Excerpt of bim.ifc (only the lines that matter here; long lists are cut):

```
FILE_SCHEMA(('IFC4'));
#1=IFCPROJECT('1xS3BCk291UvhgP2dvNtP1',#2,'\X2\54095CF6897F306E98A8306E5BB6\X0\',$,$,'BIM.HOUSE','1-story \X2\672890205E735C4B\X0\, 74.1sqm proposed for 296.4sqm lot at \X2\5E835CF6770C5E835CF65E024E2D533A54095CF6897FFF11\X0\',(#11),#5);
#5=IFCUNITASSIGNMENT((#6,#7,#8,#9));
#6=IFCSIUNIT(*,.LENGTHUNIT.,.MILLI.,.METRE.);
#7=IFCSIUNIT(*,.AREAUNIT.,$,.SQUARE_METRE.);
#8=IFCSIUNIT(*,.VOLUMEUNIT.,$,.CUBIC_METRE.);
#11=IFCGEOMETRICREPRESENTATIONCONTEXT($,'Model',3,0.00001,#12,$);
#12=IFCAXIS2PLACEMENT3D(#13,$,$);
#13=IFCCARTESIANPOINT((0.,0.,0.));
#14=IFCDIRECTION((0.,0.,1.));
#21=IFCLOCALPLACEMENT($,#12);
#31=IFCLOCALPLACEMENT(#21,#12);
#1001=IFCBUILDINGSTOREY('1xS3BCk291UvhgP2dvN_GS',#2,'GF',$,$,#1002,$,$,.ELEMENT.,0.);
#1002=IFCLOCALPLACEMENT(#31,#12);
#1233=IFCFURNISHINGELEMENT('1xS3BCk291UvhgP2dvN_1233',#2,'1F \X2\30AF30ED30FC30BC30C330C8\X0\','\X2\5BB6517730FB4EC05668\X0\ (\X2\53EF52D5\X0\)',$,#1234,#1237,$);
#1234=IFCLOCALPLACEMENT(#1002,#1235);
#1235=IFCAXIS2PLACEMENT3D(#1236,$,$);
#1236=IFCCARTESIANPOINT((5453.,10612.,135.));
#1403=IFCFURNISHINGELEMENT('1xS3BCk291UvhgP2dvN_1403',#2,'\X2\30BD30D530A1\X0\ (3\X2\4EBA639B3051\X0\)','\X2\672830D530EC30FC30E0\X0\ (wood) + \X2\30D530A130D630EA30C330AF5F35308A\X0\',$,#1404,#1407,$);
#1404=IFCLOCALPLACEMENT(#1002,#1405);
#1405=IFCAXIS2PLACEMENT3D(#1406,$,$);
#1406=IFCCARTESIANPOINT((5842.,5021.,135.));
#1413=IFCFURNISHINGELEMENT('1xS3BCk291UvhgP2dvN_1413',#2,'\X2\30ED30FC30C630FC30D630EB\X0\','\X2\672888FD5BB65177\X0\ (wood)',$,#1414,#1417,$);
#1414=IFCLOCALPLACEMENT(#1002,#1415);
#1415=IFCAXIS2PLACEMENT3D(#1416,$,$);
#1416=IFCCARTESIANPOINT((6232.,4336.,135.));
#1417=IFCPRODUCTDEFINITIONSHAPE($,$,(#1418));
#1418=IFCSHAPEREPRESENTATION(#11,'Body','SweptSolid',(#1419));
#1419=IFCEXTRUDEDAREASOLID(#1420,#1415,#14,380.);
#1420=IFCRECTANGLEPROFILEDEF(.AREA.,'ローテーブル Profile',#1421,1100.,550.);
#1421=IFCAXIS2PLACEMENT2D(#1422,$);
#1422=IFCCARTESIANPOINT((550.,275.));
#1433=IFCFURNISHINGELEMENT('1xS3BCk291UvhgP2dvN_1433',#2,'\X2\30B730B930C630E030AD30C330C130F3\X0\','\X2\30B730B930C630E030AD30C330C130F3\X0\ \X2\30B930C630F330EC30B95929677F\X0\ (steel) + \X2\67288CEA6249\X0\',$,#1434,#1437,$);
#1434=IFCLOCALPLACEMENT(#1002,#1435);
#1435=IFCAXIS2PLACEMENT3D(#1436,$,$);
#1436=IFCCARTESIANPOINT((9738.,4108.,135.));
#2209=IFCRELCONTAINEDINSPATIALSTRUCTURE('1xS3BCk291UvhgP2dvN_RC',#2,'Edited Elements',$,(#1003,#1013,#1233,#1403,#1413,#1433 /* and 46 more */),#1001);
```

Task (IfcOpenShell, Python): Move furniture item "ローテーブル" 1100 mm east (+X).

```python
import ifcopenshell
import ifcopenshell.api.geometry
import ifcopenshell.util.placement
import ifcopenshell.util.unit

model = ifcopenshell.open("bim.ifc")
unit_scale = ifcopenshell.util.unit.calculate_unit_scale(model)

item = model.by_id(1413)
matrix = ifcopenshell.util.placement.get_local_placement(item.ObjectPlacement)
matrix[0, 3] += 1.1 / unit_scale
ifcopenshell.api.geometry.edit_object_placement(model, product=item, matrix=matrix, is_si=False)

print(ifcopenshell.util.placement.get_local_placement(item.ObjectPlacement).round(3) + 0.0)

model.write("bim_updated.ifc")
```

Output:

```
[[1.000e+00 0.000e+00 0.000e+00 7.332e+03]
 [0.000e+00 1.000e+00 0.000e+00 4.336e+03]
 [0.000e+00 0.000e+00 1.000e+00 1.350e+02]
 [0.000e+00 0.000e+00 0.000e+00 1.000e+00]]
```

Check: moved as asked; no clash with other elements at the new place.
